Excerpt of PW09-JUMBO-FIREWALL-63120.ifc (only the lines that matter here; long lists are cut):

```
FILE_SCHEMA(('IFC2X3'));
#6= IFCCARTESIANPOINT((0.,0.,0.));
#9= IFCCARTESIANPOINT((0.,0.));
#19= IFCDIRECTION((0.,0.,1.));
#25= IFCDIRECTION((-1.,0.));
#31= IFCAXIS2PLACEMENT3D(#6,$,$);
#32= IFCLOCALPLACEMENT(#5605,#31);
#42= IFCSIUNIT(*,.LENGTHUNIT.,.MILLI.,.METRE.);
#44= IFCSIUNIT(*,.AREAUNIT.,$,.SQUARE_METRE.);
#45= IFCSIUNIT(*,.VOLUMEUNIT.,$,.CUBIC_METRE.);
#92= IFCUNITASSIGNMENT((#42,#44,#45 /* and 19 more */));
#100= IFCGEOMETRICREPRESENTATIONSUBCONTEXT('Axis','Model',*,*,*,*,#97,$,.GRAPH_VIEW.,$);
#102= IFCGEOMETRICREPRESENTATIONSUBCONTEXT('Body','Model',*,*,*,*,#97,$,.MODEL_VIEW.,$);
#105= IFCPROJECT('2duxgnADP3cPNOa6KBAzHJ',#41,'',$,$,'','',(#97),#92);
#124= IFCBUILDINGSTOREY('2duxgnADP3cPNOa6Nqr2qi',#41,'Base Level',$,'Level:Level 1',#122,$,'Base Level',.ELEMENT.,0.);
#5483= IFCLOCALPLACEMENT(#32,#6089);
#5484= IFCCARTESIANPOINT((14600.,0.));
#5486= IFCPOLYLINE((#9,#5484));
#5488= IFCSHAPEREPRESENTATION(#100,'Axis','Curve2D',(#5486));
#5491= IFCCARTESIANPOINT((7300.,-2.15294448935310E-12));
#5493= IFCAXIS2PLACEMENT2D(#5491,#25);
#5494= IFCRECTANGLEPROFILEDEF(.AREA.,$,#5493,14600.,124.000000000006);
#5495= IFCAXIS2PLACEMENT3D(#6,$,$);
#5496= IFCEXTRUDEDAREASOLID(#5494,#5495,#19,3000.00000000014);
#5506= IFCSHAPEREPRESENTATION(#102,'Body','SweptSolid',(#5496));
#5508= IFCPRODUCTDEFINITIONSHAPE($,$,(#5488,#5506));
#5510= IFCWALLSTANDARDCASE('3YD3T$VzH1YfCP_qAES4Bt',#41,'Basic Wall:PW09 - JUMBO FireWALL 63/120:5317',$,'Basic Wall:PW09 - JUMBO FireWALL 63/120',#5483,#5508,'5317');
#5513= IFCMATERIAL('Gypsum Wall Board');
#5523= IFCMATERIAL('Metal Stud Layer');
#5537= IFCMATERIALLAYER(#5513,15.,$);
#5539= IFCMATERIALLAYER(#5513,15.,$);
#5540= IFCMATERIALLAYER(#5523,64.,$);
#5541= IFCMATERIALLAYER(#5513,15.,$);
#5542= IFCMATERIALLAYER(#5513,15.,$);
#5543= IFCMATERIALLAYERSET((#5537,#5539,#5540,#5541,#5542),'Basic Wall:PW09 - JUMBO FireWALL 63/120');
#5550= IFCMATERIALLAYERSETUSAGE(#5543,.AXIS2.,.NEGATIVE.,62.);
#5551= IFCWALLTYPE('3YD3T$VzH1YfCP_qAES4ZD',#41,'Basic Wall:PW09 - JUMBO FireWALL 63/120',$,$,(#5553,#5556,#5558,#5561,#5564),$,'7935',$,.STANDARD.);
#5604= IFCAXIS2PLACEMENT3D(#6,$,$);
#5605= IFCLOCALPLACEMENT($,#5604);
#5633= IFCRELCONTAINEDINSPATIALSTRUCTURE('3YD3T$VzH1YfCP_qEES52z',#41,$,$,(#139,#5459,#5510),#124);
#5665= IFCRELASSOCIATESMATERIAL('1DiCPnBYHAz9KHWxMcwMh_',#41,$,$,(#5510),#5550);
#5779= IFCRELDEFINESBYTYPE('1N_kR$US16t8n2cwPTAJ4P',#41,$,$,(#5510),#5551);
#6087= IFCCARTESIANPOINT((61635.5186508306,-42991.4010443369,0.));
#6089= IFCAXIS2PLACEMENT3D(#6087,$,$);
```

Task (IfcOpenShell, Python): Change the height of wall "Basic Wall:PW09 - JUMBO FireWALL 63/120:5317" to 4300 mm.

```python
import ifcopenshell
import ifcopenshell.geom
import ifcopenshell.util.representation
import ifcopenshell.util.shape
import ifcopenshell.util.unit

model = ifcopenshell.open("PW09-JUMBO-FIREWALL-63120.ifc")
unit_scale = ifcopenshell.util.unit.calculate_unit_scale(model)
settings = ifcopenshell.geom.settings()


def volume(element):
    """Net volume in cubic metres, openings subtracted."""
    shape = ifcopenshell.geom.create_shape(settings, element)
    return ifcopenshell.util.shape.get_volume(shape.geometry)


wall = model.by_id(5510)
before = volume(wall)

body = ifcopenshell.util.representation.get_representation(wall, "Model", "Body")
solid = body.Items[0]
old_height = solid.Depth
solid.Depth = 4.3 / unit_scale
after = volume(wall)

print(f"height {old_height:g} -> {solid.Depth:g}, volume {before:.3f} -> {after:.3f} m3")

model.write("PW09-JUMBO-FIREWALL-63120_v2.ifc")
```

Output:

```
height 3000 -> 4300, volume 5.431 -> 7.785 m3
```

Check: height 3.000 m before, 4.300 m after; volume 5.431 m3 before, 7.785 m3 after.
